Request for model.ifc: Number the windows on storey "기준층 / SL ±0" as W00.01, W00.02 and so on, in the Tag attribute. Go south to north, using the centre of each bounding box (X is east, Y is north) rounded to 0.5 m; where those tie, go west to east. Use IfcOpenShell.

First a look at what the model holds.

```python
import ifcopenshell
import ifcopenshell.util.element
import ifcopenshell.util.placement

model = ifcopenshell.open("model.ifc")
print(model.schema)
storey = next(s for s in model.by_type("IfcBuildingStorey") if s.Name == "기준층 / SL ±0")
windows = [e for e in ifcopenshell.util.element.get_decomposition(storey) if e.is_a("IfcWindow")]
for e in sorted(windows, key=lambda e: e.id()):
    origin = ifcopenshell.util.placement.get_local_placement(e.ObjectPlacement)[:3, 3]
    print(e.id(), e.Tag, e.Name, origin.round(2) + 0.0, sep=" | ")
```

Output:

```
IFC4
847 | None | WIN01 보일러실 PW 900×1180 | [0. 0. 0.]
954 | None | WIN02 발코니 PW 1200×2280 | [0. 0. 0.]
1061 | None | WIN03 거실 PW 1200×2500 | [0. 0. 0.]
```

```python
import ifcopenshell
import ifcopenshell.geom
import ifcopenshell.util.element
import ifcopenshell.util.shape

model = ifcopenshell.open("model.ifc")
settings = ifcopenshell.geom.settings()
settings.set("use-world-coords", True)


def centre(element):
    shape = ifcopenshell.geom.create_shape(settings, element)
    return ifcopenshell.util.shape.get_bbox_centroid(shape.geometry)


storey = next(s for s in model.by_type("IfcBuildingStorey") if s.Name == "기준층 / SL ±0")
windows = [e for e in ifcopenshell.util.element.get_decomposition(storey) if e.is_a("IfcWindow")]

# Insertion points can sit at a corner or the storey origin, so sort by the geometry (in metres).
centres = {e: centre(e) for e in windows}
windows.sort(key=lambda e: (round(centres[e][1] / 0.5), centres[e][0]))

for i, e in enumerate(windows, start=1):
    number = f"W00.{i:02d}"
    e.Tag = number
    print(e.id(), number)

model.write("model_v2.ifc")
```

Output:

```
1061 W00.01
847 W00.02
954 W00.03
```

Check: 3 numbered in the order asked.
